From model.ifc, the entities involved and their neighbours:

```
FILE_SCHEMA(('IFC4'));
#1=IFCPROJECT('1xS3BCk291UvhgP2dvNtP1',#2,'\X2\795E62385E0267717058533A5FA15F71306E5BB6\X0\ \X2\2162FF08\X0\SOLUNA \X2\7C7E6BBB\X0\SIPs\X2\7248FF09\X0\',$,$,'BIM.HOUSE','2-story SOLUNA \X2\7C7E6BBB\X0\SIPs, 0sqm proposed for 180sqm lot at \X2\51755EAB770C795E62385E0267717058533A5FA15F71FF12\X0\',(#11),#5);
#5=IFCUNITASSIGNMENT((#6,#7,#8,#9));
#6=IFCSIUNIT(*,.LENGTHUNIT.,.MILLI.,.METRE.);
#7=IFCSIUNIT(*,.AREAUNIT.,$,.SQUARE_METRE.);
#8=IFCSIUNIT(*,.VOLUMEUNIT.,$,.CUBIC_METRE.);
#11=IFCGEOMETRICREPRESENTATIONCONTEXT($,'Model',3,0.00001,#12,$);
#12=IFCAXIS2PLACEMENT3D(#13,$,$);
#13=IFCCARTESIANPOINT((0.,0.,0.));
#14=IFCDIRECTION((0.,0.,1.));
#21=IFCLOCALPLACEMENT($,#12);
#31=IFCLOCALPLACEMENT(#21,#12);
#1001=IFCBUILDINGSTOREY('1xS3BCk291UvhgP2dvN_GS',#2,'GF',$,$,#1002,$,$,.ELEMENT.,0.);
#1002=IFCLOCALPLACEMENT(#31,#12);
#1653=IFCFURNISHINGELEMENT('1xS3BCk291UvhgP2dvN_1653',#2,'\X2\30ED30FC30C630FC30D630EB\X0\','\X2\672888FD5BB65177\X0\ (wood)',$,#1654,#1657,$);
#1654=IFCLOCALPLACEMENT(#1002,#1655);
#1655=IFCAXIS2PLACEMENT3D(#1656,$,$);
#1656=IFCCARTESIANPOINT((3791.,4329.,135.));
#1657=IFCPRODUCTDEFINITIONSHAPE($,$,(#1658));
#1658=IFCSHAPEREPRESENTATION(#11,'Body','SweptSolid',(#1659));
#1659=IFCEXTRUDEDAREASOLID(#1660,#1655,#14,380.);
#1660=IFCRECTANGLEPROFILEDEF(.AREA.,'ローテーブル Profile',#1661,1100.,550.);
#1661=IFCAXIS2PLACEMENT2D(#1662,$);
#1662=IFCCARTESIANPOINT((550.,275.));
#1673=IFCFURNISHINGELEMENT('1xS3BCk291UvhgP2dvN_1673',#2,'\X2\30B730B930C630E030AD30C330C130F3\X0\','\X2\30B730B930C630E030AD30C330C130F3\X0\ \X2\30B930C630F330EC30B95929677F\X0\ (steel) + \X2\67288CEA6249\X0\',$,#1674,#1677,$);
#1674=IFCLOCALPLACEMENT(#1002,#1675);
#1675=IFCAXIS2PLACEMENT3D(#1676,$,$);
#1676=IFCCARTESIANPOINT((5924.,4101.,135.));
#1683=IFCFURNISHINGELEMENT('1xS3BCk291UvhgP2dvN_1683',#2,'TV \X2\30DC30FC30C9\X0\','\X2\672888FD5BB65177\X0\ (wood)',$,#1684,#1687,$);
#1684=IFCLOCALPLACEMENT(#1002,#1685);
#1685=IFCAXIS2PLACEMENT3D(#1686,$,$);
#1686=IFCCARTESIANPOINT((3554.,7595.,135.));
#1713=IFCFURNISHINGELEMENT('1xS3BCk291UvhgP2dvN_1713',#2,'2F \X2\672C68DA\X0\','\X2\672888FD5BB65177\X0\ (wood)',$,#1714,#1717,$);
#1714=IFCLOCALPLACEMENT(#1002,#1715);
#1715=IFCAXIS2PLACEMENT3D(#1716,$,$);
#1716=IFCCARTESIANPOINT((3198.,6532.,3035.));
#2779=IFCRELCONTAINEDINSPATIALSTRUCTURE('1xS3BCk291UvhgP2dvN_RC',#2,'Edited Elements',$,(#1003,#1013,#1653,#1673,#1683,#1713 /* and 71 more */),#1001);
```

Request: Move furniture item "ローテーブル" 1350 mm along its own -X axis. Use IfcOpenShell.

```python
import ifcopenshell
import ifcopenshell.api.geometry
import ifcopenshell.util.placement
import ifcopenshell.util.unit

model = ifcopenshell.open("model.ifc")
unit_scale = ifcopenshell.util.unit.calculate_unit_scale(model)

item = model.by_guid("1xS3BCk291UvhgP2dvN_1653")
matrix = ifcopenshell.util.placement.get_local_placement(item.ObjectPlacement)
matrix[:3, 3] -= matrix[:3, 0] * 1.35 / unit_scale
ifcopenshell.api.geometry.edit_object_placement(model, product=item, matrix=matrix, is_si=False)

print(ifcopenshell.util.placement.get_local_placement(item.ObjectPlacement).round(3) + 0.0)

model.write("model_edited.ifc")
```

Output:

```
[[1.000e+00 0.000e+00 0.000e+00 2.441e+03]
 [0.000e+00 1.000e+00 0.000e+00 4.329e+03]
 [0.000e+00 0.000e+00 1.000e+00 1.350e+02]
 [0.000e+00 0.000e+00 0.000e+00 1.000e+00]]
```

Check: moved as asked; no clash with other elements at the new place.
